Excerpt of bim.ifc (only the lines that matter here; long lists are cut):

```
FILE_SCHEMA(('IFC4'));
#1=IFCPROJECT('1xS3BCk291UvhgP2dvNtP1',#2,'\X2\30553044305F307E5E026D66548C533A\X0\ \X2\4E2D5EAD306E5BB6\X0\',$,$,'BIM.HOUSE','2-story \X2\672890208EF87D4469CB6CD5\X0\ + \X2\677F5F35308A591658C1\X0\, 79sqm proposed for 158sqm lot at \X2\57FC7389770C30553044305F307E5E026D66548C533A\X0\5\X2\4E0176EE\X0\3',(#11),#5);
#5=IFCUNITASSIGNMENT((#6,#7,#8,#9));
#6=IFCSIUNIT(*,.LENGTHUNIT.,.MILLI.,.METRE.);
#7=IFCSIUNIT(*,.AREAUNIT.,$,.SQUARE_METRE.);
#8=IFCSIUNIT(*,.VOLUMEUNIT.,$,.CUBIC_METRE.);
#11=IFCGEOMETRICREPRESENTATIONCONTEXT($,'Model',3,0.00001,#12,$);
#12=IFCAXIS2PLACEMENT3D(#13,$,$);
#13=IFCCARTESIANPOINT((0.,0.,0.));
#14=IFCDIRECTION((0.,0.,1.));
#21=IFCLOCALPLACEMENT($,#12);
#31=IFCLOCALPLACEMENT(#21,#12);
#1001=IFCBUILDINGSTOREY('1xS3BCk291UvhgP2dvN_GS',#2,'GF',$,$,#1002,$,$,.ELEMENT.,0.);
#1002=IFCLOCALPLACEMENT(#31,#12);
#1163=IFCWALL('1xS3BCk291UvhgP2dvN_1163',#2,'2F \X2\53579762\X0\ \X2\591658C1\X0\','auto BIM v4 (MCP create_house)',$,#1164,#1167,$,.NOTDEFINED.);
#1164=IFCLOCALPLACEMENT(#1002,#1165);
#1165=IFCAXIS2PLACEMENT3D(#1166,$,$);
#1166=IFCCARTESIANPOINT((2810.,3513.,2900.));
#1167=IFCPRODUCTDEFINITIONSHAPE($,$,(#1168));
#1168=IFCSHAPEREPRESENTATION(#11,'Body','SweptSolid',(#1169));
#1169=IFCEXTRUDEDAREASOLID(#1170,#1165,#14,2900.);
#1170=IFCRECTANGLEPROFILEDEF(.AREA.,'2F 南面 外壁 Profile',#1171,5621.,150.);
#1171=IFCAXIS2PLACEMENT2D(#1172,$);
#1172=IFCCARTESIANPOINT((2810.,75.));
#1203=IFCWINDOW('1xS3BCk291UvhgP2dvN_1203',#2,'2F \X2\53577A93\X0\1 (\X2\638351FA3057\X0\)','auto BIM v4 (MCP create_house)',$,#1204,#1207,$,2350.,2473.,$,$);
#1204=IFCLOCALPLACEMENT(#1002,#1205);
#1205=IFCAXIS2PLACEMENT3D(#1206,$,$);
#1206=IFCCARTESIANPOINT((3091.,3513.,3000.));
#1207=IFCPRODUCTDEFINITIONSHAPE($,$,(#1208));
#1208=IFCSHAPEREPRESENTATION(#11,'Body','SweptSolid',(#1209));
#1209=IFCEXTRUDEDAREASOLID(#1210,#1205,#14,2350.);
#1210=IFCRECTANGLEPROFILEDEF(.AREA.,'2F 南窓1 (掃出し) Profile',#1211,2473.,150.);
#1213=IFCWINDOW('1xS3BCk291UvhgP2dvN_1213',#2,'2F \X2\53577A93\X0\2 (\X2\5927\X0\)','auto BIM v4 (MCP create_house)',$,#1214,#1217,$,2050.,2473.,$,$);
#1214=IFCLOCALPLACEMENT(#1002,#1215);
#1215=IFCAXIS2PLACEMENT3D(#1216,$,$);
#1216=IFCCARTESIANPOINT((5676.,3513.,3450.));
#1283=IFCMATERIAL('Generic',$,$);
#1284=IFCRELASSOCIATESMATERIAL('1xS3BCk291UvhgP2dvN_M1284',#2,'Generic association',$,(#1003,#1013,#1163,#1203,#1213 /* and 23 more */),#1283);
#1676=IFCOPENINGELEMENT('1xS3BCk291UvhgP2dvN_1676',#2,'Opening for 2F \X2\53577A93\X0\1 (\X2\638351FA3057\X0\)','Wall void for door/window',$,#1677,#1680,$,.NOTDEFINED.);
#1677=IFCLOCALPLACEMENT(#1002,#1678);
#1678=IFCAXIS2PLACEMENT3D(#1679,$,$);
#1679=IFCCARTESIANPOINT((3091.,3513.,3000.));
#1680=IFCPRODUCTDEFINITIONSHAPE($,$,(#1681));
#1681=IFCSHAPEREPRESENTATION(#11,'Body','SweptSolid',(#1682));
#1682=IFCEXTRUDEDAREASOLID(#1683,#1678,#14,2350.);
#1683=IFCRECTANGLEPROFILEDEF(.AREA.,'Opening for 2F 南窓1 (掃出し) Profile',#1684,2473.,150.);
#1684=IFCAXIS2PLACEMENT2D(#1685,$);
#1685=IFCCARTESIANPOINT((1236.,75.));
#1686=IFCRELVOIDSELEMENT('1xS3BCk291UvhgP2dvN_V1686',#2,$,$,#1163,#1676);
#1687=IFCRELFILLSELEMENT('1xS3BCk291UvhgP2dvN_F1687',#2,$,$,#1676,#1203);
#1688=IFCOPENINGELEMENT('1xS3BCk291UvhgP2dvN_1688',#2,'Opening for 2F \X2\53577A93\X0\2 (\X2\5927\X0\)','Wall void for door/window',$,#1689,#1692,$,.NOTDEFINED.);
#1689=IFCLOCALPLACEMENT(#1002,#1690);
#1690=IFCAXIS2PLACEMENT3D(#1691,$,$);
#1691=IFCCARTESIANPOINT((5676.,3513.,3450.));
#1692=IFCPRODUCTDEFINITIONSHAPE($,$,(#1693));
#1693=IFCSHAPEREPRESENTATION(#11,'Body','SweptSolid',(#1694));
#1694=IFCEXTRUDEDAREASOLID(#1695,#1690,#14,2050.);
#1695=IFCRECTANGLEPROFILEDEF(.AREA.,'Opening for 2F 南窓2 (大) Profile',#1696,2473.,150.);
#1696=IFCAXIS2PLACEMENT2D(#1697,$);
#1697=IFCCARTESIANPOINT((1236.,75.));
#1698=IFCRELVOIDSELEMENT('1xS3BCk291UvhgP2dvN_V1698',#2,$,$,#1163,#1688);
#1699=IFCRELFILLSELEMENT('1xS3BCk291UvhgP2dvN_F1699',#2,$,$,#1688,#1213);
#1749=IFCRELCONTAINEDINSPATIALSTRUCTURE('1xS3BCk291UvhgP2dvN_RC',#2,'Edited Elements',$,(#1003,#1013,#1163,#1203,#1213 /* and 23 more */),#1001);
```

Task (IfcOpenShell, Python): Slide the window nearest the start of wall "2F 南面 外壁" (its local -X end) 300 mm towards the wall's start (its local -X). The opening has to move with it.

```python
import ifcopenshell
import ifcopenshell.api.geometry
import ifcopenshell.util.placement
import ifcopenshell.util.unit

model = ifcopenshell.open("bim.ifc")
unit_scale = ifcopenshell.util.unit.calculate_unit_scale(model)

window = model.by_id(1203)
opening = window.FillsVoids[0].RelatingOpeningElement
wall = opening.VoidsElements[0].RelatingBuildingElement

wall_matrix = ifcopenshell.util.placement.get_local_placement(wall.ObjectPlacement)
shift = wall_matrix[:3, 0] * -0.3 / unit_scale
before = ifcopenshell.util.placement.get_local_placement(window.ObjectPlacement)[:3, 3].copy()

# The window is not placed relative to its opening, so move both.
for product in (opening, window):
    matrix = ifcopenshell.util.placement.get_local_placement(product.ObjectPlacement)
    matrix[:3, 3] += shift
    ifcopenshell.api.geometry.edit_object_placement(model, product=product, matrix=matrix, is_si=False)

after = ifcopenshell.util.placement.get_local_placement(window.ObjectPlacement)[:3, 3]
print("window moved by", (after - before).round(3) + 0.0)

model.write("bim_edited.ifc")
```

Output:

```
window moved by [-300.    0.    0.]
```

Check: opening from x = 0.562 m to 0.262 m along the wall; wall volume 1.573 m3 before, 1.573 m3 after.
